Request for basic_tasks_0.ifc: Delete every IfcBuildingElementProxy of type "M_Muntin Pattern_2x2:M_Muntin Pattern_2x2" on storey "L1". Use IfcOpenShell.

First a look at what the model holds.

```python
import ifcopenshell
import ifcopenshell.util.element

model = ifcopenshell.open("basic_tasks_0.ifc")
print(model.schema)
storey = next(s for s in model.by_type("IfcBuildingStorey") if s.Name == "L1")
proxies = [e for e in ifcopenshell.util.element.get_decomposition(storey) if e.is_a("IfcBuildingElementProxy")]
seen = {}
for e in proxies:
    element_type = ifcopenshell.util.element.get_type(e)
    name = element_type.Name if element_type not in (None, e) else None
    seen[name] = seen.get(name, 0) + 1
for name, count in sorted(seen.items(), key=str):
    print(count, "x", name)
```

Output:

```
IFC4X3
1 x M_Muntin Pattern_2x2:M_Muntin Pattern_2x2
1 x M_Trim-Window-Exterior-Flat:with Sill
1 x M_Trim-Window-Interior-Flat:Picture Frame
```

```python
import ifcopenshell
import ifcopenshell.api.root
import ifcopenshell.util.element

model = ifcopenshell.open("basic_tasks_0.ifc")

storey = next(s for s in model.by_type("IfcBuildingStorey") if s.Name == "L1")
proxies = [e for e in ifcopenshell.util.element.get_decomposition(storey) if e.is_a("IfcBuildingElementProxy")]
targets = [e for e in proxies if (t := ifcopenshell.util.element.get_type(e)) not in (None, e) and t.Name == "M_Muntin Pattern_2x2:M_Muntin Pattern_2x2"]

for e in targets:
    ifcopenshell.api.root.remove_product(model, product=e)
print(len(targets), "removed")

model.write("basic_tasks_0_v2.ifc")
```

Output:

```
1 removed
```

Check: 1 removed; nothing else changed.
